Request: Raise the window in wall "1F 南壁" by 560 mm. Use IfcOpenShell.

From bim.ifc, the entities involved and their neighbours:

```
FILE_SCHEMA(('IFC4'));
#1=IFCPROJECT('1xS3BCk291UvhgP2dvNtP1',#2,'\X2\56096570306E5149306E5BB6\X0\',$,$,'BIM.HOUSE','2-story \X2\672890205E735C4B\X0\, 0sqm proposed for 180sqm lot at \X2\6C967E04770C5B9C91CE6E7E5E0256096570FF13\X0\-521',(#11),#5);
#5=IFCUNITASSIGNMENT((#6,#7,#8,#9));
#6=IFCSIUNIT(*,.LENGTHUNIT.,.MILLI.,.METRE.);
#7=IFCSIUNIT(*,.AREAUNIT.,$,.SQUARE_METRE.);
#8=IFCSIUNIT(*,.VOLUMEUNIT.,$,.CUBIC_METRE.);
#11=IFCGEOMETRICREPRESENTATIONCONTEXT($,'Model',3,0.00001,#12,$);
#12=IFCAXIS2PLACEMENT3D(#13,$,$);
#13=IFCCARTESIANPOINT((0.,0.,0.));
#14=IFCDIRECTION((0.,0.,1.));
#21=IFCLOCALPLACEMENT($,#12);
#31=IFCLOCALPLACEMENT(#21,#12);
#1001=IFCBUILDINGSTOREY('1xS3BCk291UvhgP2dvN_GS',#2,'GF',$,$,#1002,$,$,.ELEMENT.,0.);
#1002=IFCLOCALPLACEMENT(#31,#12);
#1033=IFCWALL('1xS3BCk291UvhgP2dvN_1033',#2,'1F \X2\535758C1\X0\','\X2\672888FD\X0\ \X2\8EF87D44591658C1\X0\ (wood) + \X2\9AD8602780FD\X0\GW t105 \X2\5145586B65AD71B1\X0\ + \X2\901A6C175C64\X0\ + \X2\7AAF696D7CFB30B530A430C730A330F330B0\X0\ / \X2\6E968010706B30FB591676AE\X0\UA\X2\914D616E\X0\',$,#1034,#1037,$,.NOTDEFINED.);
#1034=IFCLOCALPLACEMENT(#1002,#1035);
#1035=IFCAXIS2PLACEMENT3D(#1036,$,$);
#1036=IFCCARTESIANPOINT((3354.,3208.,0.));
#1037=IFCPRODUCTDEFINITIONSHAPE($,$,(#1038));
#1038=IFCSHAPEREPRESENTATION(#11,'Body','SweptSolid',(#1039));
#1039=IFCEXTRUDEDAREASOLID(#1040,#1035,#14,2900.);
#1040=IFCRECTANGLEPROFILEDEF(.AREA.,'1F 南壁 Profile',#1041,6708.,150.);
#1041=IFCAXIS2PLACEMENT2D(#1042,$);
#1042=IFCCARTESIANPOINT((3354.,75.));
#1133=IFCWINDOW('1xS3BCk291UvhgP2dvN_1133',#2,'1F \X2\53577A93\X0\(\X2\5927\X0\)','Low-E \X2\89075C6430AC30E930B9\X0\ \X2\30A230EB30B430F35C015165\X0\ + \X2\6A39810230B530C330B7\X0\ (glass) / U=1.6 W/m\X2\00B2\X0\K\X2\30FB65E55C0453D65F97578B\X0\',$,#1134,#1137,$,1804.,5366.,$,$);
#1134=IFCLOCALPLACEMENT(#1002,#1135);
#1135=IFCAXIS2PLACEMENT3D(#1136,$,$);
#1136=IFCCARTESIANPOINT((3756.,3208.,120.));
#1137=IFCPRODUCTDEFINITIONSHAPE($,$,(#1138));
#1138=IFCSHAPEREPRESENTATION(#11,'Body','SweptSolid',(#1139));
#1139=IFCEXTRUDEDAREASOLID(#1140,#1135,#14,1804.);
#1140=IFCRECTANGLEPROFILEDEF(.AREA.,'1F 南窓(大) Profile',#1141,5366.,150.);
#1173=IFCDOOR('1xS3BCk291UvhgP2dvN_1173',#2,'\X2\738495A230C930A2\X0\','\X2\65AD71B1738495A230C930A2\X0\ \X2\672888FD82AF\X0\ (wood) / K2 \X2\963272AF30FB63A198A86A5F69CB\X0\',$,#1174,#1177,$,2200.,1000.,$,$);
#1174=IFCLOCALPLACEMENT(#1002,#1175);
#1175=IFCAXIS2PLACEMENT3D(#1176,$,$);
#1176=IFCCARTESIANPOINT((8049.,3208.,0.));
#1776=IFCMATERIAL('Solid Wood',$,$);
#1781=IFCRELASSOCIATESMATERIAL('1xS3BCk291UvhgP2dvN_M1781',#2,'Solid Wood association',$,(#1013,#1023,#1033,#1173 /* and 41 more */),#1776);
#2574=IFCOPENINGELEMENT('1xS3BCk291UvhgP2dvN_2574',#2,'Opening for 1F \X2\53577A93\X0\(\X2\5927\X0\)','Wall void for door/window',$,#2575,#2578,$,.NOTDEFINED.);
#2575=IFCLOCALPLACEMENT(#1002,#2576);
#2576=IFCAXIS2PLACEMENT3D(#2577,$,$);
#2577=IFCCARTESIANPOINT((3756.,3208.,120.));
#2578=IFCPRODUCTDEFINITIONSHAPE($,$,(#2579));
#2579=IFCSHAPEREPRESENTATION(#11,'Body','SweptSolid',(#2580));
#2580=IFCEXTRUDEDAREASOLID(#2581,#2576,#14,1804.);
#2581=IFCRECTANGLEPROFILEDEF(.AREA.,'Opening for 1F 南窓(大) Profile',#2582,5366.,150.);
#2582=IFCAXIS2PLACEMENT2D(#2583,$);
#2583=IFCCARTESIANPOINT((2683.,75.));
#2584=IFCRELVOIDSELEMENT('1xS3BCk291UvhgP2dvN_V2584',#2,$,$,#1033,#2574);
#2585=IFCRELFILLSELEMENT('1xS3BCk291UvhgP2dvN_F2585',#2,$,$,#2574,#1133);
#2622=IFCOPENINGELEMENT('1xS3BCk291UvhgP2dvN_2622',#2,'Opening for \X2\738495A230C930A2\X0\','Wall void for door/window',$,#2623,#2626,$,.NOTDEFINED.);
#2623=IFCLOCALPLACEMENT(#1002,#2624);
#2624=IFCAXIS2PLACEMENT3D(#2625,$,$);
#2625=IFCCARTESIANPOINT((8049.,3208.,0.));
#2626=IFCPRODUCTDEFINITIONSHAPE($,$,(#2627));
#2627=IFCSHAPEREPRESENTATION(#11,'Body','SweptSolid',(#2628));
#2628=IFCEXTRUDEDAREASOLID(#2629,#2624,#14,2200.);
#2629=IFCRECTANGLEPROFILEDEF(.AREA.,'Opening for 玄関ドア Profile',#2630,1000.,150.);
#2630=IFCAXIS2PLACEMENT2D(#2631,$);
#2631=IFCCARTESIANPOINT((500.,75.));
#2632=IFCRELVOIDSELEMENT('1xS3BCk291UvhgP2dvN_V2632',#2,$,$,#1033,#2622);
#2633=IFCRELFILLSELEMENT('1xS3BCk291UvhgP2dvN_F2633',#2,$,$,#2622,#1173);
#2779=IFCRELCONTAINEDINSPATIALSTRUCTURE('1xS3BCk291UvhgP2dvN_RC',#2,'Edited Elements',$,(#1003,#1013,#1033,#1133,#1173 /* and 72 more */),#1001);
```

```python
import numpy as np
import ifcopenshell
import ifcopenshell.api.geometry
import ifcopenshell.util.placement
import ifcopenshell.util.unit

model = ifcopenshell.open("bim.ifc")
unit_scale = ifcopenshell.util.unit.calculate_unit_scale(model)

window = model.by_guid("1xS3BCk291UvhgP2dvN_1133")
opening = window.FillsVoids[0].RelatingOpeningElement
dz = 0.56 / unit_scale

shift = np.array([0.0, 0.0, dz])
# The window is not placed relative to its opening, so move both.
for product in (opening, window):
    matrix = ifcopenshell.util.placement.get_local_placement(product.ObjectPlacement)
    matrix[:3, 3] += shift
    ifcopenshell.api.geometry.edit_object_placement(model, product=product, matrix=matrix, is_si=False)

print(f"moved by {dz * unit_scale:+.3f} m")

model.write("bim_updated.ifc")
```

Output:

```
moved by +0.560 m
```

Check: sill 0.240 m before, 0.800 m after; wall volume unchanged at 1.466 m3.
